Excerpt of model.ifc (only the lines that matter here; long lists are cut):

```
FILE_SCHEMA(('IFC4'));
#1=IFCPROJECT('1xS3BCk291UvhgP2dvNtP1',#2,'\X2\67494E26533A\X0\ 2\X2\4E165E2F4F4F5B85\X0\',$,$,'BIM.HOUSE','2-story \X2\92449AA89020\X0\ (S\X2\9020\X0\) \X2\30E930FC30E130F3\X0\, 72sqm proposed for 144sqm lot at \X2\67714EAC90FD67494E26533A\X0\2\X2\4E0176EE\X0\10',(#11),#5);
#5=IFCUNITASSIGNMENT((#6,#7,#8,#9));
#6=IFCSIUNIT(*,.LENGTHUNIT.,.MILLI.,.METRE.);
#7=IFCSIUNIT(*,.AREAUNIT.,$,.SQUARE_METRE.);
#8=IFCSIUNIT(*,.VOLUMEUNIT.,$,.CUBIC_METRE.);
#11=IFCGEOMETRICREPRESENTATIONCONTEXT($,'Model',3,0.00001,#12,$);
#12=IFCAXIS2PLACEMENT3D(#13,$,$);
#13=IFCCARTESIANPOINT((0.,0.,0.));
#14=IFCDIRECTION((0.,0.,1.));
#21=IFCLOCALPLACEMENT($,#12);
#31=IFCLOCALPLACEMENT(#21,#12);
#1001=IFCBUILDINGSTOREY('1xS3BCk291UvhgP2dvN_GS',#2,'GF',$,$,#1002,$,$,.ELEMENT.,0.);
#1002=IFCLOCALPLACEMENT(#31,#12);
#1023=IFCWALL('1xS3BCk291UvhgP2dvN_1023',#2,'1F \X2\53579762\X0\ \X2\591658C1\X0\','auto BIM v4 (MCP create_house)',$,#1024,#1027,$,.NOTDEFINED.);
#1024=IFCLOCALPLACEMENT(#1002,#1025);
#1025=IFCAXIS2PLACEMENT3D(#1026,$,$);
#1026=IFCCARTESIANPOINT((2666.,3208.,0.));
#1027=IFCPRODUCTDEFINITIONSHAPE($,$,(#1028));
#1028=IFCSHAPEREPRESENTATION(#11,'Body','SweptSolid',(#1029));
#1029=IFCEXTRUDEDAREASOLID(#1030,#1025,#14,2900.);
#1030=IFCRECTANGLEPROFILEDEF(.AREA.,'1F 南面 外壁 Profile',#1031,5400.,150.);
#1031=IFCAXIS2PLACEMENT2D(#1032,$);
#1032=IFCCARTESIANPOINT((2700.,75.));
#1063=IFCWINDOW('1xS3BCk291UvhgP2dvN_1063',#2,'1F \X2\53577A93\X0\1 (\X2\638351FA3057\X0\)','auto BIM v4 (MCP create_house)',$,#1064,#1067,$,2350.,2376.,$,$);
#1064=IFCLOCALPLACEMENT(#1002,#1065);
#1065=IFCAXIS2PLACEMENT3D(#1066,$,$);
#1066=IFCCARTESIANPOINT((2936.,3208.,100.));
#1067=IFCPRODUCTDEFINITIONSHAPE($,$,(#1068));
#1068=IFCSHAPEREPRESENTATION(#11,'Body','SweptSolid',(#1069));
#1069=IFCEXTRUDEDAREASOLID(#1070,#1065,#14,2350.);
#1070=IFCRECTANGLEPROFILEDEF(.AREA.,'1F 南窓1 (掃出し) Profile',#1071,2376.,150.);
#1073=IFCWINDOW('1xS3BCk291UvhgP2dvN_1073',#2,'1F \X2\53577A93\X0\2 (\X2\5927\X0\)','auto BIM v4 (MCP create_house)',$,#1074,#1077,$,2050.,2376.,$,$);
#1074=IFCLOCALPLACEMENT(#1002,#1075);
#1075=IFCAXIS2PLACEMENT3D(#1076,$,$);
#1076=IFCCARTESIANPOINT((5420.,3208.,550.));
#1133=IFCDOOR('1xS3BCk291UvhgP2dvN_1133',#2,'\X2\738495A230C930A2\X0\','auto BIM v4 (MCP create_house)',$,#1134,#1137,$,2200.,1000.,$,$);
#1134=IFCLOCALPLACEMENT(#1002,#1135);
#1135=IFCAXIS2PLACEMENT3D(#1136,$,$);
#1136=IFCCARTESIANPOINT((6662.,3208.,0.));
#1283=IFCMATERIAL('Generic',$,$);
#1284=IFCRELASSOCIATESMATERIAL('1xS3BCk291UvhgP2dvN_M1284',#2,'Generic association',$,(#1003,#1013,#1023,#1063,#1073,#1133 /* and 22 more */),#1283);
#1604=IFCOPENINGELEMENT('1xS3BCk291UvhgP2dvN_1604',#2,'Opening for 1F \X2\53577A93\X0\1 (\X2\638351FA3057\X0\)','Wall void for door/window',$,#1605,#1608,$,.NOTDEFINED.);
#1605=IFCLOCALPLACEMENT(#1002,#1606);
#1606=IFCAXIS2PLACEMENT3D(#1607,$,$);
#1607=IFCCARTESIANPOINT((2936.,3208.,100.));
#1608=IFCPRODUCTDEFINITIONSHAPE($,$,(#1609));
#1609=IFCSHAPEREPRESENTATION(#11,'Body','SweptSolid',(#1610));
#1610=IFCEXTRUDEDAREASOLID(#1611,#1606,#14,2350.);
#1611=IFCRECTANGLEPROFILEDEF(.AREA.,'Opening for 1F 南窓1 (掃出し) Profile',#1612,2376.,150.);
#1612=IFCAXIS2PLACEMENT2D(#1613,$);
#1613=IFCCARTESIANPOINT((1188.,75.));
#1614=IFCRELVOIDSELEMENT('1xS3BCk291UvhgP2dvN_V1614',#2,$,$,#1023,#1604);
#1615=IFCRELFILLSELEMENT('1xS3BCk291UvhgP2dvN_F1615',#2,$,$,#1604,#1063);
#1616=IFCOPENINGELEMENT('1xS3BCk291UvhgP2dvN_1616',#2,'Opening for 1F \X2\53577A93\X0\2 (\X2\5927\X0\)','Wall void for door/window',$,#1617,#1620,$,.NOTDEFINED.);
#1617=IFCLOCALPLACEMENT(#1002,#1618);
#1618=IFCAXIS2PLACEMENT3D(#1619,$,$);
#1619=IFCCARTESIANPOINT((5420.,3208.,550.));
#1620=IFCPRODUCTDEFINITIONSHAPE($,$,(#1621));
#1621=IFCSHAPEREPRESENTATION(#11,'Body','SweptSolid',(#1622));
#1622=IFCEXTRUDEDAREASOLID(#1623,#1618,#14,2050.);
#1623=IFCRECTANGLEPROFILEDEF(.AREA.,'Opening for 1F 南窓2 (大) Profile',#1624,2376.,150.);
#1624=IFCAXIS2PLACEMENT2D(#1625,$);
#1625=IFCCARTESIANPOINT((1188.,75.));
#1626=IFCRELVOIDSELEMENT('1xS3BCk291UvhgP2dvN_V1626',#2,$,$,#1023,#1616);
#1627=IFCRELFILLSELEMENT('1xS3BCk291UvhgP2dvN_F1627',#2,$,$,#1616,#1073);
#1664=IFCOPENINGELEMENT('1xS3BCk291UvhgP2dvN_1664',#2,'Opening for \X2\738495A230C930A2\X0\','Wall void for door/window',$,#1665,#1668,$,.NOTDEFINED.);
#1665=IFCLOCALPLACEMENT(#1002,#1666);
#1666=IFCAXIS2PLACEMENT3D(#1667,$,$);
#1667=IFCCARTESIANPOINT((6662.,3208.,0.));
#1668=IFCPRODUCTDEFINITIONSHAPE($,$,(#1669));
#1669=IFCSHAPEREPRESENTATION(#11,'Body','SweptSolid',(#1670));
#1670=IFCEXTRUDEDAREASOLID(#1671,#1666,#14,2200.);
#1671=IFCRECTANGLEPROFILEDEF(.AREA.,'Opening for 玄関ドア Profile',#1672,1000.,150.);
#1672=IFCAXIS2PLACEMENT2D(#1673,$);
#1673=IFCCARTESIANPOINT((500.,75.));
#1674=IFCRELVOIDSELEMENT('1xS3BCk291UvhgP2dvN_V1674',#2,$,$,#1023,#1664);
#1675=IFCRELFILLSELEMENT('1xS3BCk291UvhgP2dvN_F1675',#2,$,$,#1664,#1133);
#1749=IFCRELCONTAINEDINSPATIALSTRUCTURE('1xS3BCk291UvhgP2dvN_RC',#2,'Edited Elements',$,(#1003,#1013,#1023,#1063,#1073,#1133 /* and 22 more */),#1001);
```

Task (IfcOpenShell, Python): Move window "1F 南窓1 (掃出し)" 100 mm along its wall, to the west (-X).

```python
import ifcopenshell
import ifcopenshell.api.geometry
import ifcopenshell.util.placement

model = ifcopenshell.open("model.ifc")

window = model.by_guid("1xS3BCk291UvhgP2dvN_1063")
opening = window.FillsVoids[0].RelatingOpeningElement
wall = opening.VoidsElements[0].RelatingBuildingElement

wall_matrix = ifcopenshell.util.placement.get_local_placement(wall.ObjectPlacement)
shift = wall_matrix[:3, 0] * -100.0
before = ifcopenshell.util.placement.get_local_placement(window.ObjectPlacement)[:3, 3].copy()

# The window is not placed relative to its opening, so move both.
for product in (opening, window):
    matrix = ifcopenshell.util.placement.get_local_placement(product.ObjectPlacement)
    matrix[:3, 3] += shift
    ifcopenshell.api.geometry.edit_object_placement(model, product=product, matrix=matrix, is_si=False)

after = ifcopenshell.util.placement.get_local_placement(window.ObjectPlacement)[:3, 3]
print("window moved by", (after - before).round(3) + 0.0)

model.write("model_edited.ifc")
```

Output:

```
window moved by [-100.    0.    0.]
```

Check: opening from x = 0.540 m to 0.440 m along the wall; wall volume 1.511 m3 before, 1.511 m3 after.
